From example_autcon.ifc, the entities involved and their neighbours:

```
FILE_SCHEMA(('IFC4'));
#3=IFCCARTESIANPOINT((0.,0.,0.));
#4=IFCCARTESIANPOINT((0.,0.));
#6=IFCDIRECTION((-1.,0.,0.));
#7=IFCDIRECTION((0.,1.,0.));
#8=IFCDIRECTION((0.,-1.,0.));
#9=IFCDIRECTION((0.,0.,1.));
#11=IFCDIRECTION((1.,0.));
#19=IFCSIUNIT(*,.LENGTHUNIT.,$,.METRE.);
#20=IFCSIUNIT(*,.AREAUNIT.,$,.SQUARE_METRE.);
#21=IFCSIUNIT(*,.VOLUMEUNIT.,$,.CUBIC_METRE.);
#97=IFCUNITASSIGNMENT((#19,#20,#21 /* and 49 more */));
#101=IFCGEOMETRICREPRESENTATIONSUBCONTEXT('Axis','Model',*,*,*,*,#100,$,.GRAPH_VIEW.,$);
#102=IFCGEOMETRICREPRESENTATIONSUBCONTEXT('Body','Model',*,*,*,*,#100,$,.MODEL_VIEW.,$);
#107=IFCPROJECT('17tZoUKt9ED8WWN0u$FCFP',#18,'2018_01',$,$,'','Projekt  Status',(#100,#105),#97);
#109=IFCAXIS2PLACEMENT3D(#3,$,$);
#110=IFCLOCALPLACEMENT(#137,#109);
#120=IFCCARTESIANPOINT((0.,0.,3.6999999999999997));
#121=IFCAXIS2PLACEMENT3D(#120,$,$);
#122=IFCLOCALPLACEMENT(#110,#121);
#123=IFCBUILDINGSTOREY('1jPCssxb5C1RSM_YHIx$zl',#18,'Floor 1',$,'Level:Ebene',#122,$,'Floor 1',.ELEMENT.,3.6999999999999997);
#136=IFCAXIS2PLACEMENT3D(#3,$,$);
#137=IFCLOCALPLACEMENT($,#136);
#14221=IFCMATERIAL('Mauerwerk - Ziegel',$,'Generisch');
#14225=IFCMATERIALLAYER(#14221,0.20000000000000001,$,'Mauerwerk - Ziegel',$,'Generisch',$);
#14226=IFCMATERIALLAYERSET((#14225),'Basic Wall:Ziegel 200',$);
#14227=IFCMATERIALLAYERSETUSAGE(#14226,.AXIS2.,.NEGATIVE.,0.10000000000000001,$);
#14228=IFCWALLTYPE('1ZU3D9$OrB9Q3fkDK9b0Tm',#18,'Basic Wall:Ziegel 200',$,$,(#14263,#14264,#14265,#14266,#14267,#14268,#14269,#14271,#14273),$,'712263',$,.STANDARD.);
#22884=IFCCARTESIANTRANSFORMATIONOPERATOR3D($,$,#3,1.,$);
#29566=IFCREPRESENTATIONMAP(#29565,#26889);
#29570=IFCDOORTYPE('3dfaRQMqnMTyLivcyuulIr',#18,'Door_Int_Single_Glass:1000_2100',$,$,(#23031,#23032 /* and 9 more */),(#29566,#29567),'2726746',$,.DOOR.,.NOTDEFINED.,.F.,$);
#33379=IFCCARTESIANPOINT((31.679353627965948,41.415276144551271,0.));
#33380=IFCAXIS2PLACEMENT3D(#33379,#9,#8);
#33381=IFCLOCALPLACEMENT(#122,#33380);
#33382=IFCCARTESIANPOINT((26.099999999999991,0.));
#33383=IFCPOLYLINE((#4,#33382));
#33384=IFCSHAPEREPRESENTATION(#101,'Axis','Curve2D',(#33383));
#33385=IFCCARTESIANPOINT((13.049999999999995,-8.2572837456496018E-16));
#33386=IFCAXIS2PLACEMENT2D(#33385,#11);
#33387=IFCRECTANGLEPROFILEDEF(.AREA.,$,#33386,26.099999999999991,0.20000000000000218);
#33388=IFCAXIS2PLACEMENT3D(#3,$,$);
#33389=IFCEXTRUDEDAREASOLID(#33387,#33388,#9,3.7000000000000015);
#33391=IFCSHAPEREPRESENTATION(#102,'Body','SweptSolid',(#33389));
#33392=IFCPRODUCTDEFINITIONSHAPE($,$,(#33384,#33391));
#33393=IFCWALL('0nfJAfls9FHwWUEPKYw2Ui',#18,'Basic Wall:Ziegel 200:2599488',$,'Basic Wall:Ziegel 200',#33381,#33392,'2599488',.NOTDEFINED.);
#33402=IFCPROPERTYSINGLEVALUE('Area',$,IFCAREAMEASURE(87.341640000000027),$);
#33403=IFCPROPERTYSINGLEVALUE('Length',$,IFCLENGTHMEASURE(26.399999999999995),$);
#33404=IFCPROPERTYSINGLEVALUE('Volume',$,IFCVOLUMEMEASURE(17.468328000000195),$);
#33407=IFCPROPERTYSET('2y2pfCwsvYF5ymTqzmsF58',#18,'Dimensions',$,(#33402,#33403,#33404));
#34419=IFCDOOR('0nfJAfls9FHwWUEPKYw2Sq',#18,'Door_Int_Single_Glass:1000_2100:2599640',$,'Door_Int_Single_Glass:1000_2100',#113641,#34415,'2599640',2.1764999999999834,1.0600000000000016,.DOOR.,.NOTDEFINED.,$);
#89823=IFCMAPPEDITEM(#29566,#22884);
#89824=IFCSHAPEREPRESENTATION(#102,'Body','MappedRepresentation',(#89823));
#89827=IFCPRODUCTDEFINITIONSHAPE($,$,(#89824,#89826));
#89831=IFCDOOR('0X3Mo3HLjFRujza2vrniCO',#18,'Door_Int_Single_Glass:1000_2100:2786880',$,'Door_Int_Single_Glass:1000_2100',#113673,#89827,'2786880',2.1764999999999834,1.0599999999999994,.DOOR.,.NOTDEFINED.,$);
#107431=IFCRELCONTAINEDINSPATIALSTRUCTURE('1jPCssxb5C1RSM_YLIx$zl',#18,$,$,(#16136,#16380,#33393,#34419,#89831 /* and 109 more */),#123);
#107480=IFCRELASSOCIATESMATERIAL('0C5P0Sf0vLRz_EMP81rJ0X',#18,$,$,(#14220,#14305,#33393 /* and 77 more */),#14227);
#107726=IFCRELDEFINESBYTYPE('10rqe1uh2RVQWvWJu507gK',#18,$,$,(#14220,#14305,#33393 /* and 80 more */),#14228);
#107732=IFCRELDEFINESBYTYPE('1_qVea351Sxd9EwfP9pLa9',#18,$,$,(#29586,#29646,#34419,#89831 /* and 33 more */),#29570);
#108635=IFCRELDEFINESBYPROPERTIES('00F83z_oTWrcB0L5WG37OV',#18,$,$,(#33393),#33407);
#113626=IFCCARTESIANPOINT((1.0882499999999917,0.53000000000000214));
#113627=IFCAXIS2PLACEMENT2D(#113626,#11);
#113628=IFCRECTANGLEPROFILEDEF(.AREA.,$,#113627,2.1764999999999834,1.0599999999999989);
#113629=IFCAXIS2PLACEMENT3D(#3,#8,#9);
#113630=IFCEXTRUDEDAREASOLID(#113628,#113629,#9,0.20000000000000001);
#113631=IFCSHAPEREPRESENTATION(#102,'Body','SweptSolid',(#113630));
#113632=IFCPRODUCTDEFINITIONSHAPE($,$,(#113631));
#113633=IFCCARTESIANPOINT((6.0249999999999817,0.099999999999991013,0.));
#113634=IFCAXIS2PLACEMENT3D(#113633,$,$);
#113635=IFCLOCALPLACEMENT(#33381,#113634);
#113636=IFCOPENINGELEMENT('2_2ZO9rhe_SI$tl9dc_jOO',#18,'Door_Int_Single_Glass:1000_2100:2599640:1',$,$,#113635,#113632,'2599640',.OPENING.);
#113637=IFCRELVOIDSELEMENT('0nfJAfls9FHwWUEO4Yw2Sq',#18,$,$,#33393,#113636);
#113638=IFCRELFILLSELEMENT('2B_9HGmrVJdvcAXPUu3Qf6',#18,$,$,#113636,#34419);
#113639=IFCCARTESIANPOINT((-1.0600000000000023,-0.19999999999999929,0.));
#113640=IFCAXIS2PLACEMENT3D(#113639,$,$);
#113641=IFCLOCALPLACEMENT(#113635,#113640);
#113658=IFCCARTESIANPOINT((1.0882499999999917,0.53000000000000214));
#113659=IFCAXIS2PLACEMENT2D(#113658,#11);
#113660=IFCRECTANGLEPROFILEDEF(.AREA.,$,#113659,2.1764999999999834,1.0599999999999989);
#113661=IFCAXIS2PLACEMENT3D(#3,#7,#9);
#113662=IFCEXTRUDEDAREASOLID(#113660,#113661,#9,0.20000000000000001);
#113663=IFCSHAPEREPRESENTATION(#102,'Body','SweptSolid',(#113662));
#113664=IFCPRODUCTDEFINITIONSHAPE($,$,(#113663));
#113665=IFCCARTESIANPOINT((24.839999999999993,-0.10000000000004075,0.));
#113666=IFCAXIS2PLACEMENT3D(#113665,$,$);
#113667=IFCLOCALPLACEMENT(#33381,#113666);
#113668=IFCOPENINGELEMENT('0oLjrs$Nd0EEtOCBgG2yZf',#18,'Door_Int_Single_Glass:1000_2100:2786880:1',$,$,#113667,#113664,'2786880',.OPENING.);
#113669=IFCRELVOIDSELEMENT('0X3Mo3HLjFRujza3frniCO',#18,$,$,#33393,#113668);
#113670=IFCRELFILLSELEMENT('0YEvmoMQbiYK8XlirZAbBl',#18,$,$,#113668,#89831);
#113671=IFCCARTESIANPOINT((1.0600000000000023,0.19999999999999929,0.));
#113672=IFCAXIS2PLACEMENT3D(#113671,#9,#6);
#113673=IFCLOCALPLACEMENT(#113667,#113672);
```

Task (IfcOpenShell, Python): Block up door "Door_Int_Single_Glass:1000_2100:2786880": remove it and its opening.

```python
import ifcopenshell
import ifcopenshell.api.feature
import ifcopenshell.api.pset
import ifcopenshell.api.root
import ifcopenshell.geom
import ifcopenshell.util.element
import ifcopenshell.util.shape
import ifcopenshell.util.unit

model = ifcopenshell.open("example_autcon.ifc")
area_scale = ifcopenshell.util.unit.calculate_unit_scale(model, "AREAUNIT")
volume_scale = ifcopenshell.util.unit.calculate_unit_scale(model, "VOLUMEUNIT")
settings = ifcopenshell.geom.settings()


def volume(element):
    """Net volume in cubic metres, openings subtracted."""
    shape = ifcopenshell.geom.create_shape(settings, element)
    return ifcopenshell.util.shape.get_volume(shape.geometry)


door = model.by_guid("0X3Mo3HLjFRujza2vrniCO")
opening = door.FillsVoids[0].RelatingOpeningElement
wall = opening.VoidsElements[0].RelatingBuildingElement
before = volume(wall)

ifcopenshell.api.root.remove_product(model, product=door)
ifcopenshell.api.feature.remove_feature(model, feature=opening)

after = volume(wall)
thickness = 0.2  # wall thickness in metres

# Update the wall's stored quantities.
pset = model.by_id(ifcopenshell.util.element.get_pset(wall, "Dimensions", should_inherit=False)["id"])
ifcopenshell.api.pset.edit_pset(model, pset=pset, properties={
    "Area": model.create_entity("IfcAreaMeasure", after / thickness / area_scale),
    "Volume": model.create_entity("IfcVolumeMeasure", after / volume_scale),
})

print(f"wall volume {before:.3f} -> {after:.3f} m3")

model.write("example_autcon_v2.ifc")
```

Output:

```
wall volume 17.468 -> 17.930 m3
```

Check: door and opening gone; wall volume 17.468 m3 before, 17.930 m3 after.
